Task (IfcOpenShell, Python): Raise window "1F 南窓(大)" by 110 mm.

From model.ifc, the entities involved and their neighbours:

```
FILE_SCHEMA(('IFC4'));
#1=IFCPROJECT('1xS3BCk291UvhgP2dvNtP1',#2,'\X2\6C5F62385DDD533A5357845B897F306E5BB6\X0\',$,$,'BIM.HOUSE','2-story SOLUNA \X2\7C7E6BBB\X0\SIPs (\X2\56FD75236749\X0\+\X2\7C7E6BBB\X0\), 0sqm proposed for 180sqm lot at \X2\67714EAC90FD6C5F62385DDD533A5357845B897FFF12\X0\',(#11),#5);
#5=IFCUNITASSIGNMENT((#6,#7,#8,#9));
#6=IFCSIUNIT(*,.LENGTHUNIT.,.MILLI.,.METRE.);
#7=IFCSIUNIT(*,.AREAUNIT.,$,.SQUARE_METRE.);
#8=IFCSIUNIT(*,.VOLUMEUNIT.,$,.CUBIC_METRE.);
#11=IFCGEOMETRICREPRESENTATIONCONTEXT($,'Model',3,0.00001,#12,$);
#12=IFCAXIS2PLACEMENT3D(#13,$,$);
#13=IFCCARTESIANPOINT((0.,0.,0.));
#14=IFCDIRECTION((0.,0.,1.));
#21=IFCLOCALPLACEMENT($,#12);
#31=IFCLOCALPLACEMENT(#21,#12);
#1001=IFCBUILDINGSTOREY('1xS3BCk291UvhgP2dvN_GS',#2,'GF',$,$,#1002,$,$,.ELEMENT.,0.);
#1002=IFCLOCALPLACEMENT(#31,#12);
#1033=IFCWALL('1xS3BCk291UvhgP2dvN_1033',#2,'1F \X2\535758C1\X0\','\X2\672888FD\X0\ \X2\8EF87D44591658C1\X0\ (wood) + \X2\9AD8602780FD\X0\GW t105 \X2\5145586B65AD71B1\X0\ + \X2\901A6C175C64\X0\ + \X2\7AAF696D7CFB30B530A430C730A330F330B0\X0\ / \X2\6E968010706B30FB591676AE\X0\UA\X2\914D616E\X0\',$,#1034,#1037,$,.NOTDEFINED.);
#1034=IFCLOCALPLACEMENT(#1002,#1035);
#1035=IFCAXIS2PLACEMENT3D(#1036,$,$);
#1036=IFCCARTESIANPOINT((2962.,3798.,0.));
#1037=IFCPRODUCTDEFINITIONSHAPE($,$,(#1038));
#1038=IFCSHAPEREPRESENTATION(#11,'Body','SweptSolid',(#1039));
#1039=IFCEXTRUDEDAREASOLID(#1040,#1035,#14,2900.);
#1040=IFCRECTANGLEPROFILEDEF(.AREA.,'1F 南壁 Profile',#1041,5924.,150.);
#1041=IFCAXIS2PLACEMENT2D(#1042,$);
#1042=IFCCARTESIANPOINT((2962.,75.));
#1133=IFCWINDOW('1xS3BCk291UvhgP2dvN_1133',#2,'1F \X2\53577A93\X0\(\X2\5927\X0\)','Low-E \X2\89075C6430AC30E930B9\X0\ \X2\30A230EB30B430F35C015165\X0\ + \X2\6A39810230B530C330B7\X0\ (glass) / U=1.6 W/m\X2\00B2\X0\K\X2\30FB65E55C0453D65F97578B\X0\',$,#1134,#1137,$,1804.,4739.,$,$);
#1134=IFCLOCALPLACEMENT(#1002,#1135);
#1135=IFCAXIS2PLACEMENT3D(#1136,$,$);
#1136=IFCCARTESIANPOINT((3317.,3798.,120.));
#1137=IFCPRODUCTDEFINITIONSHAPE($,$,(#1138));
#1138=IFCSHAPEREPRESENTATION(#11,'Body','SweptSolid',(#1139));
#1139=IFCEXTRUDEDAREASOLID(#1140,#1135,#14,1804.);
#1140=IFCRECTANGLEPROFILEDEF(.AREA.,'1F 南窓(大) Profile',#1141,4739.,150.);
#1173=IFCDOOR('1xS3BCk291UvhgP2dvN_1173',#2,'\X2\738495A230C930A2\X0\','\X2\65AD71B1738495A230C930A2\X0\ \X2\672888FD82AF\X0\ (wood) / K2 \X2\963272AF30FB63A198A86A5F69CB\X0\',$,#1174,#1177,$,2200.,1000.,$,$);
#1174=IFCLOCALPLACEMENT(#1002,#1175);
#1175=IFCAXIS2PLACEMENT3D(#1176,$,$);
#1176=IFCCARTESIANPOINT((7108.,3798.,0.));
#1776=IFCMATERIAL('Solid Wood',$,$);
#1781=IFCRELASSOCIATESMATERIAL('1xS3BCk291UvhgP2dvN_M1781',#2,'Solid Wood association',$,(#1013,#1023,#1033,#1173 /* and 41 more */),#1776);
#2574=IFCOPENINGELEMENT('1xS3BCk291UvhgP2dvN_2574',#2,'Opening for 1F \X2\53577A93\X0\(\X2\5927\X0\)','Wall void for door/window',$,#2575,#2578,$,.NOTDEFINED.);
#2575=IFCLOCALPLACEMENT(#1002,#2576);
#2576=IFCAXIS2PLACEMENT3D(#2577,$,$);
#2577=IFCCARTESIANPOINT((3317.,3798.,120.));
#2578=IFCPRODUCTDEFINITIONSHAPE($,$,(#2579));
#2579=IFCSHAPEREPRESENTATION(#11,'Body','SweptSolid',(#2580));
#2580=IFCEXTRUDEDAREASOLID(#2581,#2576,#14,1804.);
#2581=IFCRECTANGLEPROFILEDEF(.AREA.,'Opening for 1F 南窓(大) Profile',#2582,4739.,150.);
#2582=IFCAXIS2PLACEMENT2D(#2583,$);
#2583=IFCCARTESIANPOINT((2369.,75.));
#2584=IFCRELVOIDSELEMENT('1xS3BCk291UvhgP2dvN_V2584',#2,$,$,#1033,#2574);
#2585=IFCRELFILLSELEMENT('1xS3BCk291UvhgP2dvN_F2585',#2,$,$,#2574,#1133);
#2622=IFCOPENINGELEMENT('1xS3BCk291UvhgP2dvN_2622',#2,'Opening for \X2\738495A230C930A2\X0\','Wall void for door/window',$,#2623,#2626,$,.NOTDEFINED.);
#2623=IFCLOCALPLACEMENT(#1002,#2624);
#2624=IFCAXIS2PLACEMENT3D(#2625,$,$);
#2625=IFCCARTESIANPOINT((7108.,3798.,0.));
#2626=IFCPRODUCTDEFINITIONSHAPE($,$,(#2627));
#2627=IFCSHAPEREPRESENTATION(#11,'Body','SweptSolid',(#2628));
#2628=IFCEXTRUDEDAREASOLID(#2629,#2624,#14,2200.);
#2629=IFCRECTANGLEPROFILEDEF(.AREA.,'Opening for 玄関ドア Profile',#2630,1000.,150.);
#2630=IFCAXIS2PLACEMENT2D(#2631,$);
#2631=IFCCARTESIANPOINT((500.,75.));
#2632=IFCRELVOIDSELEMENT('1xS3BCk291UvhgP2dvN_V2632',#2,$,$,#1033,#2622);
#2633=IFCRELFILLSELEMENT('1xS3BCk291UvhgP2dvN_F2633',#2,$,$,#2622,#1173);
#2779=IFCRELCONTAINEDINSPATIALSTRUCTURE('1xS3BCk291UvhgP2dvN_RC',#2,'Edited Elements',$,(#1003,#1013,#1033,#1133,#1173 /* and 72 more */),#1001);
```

```python
import numpy as np
import ifcopenshell
import ifcopenshell.api.geometry
import ifcopenshell.util.placement
import ifcopenshell.util.unit

model = ifcopenshell.open("model.ifc")
unit_scale = ifcopenshell.util.unit.calculate_unit_scale(model)

window = model.by_guid("1xS3BCk291UvhgP2dvN_1133")
opening = window.FillsVoids[0].RelatingOpeningElement
dz = 0.11 / unit_scale

shift = np.array([0.0, 0.0, dz])
# The window is not placed relative to its opening, so move both.
for product in (opening, window):
    matrix = ifcopenshell.util.placement.get_local_placement(product.ObjectPlacement)
    matrix[:3, 3] += shift
    ifcopenshell.api.geometry.edit_object_placement(model, product=product, matrix=matrix, is_si=False)

print(f"moved by {dz * unit_scale:+.3f} m")

model.write("model-out.ifc")
```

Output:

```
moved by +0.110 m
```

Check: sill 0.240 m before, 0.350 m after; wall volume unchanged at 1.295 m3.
